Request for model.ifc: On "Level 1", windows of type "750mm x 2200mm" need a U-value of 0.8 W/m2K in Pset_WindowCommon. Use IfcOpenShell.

First a look at what the model holds.

```python
import ifcopenshell
import ifcopenshell.util.element

model = ifcopenshell.open("model.ifc")
print(model.schema)
storey = next(s for s in model.by_type("IfcBuildingStorey") if s.Name == "Level 1")
windows = [e for e in ifcopenshell.util.element.get_decomposition(storey) if e.is_a("IfcWindow")]
seen = {}
for e in windows:
    element_type = ifcopenshell.util.element.get_type(e)
    key = (element_type.Name if element_type != e and element_type else None, ifcopenshell.util.element.get_pset(e, "Pset_WindowCommon", "ThermalTransmittance"))
    seen[key] = seen.get(key, 0) + 1
for (name, value), count in sorted(seen.items(), key=str):
    print(count, "x", name, "|", value)
```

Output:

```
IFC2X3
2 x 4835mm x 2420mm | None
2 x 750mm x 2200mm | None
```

```python
import ifcopenshell
import ifcopenshell.api.pset
import ifcopenshell.util.element

model = ifcopenshell.open("model.ifc")

storey = next(s for s in model.by_type("IfcBuildingStorey") if s.Name == "Level 1")
windows = [e for e in ifcopenshell.util.element.get_decomposition(storey) if e.is_a("IfcWindow")]

count = 0
for e in windows:
    element_type = ifcopenshell.util.element.get_type(e)
    if element_type in (None, e) or element_type.Name != "750mm x 2200mm":
        continue
    # add_pset returns the element's existing set when there is one.
    pset = ifcopenshell.api.pset.add_pset(model, product=e, name="Pset_WindowCommon")
    ifcopenshell.api.pset.edit_pset(model, pset=pset, properties={"ThermalTransmittance": 0.8})
    count += 1

print(count, "windows updated")

model.write("model_edited.ifc")
```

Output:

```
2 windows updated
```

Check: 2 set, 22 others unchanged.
